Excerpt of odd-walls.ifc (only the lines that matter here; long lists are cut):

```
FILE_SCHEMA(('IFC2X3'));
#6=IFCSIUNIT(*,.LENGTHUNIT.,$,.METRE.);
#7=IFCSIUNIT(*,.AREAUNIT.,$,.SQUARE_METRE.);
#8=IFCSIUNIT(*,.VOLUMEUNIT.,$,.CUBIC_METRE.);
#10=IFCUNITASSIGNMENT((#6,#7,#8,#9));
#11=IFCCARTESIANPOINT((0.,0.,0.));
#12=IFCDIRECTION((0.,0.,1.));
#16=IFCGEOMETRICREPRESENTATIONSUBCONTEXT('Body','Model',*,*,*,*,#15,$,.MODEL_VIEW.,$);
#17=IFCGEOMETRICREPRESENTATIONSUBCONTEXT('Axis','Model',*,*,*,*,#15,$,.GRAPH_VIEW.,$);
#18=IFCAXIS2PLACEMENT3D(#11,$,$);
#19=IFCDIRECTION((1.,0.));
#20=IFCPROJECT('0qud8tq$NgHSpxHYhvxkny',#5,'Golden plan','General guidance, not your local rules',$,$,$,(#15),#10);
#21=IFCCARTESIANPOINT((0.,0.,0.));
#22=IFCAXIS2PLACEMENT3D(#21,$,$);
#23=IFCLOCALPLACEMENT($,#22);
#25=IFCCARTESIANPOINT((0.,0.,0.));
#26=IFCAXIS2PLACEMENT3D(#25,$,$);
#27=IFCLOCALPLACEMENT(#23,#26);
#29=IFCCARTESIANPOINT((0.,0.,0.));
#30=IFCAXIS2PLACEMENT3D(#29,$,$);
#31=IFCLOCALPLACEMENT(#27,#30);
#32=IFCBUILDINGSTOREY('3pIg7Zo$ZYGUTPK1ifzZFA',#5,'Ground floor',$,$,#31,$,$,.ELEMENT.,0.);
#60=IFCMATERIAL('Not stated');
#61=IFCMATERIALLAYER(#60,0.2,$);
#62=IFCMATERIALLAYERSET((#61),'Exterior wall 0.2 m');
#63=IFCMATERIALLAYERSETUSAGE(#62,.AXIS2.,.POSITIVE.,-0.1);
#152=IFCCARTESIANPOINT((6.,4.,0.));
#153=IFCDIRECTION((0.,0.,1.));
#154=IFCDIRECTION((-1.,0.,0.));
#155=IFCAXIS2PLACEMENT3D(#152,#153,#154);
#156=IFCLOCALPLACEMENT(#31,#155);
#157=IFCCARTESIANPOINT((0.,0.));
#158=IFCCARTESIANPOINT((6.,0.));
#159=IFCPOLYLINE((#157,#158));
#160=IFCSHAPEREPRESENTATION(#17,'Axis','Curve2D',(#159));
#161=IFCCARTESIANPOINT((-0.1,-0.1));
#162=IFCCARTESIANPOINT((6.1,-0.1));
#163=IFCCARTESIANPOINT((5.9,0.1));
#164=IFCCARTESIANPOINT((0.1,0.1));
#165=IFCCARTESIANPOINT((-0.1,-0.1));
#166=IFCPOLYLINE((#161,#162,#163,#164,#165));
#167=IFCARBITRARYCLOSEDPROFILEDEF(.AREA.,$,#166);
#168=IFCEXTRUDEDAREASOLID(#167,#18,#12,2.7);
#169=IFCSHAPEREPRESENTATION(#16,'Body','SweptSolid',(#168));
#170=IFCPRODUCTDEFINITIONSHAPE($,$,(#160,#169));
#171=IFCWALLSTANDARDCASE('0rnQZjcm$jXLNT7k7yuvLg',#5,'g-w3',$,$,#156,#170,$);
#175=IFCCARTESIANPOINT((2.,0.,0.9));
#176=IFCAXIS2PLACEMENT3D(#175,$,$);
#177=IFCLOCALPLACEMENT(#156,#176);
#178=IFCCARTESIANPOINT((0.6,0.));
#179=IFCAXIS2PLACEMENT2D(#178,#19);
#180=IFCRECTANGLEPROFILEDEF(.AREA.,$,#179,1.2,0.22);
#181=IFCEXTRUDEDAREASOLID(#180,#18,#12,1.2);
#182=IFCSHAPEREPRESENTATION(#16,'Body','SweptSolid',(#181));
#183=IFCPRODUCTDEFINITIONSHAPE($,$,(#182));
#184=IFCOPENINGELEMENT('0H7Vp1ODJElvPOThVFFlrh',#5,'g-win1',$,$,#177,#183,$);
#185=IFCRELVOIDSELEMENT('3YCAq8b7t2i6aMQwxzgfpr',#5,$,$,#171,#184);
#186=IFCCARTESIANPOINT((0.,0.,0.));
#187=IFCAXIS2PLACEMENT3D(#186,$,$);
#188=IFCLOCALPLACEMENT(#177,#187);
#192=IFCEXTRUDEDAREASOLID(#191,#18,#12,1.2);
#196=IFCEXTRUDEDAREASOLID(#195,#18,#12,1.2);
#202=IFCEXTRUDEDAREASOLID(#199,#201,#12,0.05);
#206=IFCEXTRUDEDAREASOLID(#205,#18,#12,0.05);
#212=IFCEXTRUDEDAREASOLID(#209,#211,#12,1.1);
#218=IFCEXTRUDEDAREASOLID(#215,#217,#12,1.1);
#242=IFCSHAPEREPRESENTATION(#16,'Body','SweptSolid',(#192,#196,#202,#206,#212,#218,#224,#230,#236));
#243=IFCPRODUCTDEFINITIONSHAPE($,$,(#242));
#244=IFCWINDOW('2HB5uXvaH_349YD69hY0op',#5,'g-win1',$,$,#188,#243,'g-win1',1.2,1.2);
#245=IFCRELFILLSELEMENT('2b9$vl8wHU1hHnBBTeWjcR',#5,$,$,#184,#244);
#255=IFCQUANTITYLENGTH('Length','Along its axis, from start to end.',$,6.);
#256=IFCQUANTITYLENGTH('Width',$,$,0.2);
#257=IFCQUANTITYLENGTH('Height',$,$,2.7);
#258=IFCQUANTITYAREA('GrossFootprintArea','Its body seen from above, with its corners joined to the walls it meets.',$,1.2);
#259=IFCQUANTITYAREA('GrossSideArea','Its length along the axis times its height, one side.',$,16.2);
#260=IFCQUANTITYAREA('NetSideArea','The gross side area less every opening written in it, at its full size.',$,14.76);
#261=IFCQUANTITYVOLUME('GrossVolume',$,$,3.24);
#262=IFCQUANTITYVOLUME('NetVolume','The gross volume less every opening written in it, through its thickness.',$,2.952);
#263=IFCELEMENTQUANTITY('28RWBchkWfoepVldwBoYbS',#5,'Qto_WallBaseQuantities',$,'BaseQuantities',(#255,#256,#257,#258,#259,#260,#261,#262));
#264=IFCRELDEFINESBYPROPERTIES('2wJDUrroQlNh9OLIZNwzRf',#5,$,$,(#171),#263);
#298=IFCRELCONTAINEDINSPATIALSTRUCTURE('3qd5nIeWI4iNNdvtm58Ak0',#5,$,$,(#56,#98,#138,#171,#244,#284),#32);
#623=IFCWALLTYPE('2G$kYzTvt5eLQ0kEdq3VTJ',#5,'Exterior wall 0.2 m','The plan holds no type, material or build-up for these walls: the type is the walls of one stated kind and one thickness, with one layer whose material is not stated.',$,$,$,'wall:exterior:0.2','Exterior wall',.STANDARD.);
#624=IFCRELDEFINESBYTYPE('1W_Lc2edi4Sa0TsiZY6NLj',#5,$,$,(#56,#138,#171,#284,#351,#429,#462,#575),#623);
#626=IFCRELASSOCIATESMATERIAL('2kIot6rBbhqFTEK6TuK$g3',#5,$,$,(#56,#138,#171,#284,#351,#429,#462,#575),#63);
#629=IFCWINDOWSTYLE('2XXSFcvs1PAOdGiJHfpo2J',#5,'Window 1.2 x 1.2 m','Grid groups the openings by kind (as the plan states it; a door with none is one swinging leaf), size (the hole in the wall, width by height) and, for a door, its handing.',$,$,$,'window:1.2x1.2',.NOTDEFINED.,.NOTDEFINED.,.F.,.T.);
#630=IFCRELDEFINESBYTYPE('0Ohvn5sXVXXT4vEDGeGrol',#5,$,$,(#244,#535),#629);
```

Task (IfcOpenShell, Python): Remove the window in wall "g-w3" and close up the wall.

```python
import ifcopenshell
import ifcopenshell.api.feature
import ifcopenshell.api.pset
import ifcopenshell.api.root
import ifcopenshell.geom
import ifcopenshell.util.element
import ifcopenshell.util.shape
import ifcopenshell.util.unit

model = ifcopenshell.open("odd-walls.ifc")
area_scale = ifcopenshell.util.unit.calculate_unit_scale(model, "AREAUNIT")
volume_scale = ifcopenshell.util.unit.calculate_unit_scale(model, "VOLUMEUNIT")
settings = ifcopenshell.geom.settings()


def volume(element):
    """Net volume in cubic metres, openings subtracted."""
    shape = ifcopenshell.geom.create_shape(settings, element)
    return ifcopenshell.util.shape.get_volume(shape.geometry)


window = model.by_guid("2HB5uXvaH_349YD69hY0op")
opening = window.FillsVoids[0].RelatingOpeningElement
wall = opening.VoidsElements[0].RelatingBuildingElement
before = volume(wall)

ifcopenshell.api.root.remove_product(model, product=window)
ifcopenshell.api.feature.remove_feature(model, feature=opening)

after = volume(wall)
thickness = 0.2  # wall thickness in metres

# Update the wall's stored quantities.
qto = model.by_id(ifcopenshell.util.element.get_pset(wall, "Qto_WallBaseQuantities", should_inherit=False)["id"])
ifcopenshell.api.pset.edit_qto(model, qto=qto, properties={
    "NetSideArea": after / thickness / area_scale,
    "NetVolume": after / volume_scale,
})

print(f"wall volume {before:.3f} -> {after:.3f} m3")

model.write("odd-walls_edited.ifc")
```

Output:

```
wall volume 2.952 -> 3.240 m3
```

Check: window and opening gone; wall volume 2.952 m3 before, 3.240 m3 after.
